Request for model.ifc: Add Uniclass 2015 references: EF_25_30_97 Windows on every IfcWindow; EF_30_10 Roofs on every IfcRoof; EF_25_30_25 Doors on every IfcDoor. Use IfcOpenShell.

First a look at what the model holds.

```python
import ifcopenshell

model = ifcopenshell.open("model.ifc")
print(model.schema)
print("classifications:", [c.Name for c in model.by_type("IfcClassification")])
for ifc_class in ("IfcDoor", "IfcRoof", "IfcStair", "IfcWall", "IfcWindow"):
    print(ifc_class, len(model.by_type(ifc_class)))
```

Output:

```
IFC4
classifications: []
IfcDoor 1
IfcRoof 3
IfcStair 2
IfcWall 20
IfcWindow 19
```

```python
import ifcopenshell
import ifcopenshell.api.classification

model = ifcopenshell.open("model.ifc")

system = ifcopenshell.api.classification.add_classification(model, classification="Uniclass 2015")

codes = {
    "IfcWindow": ("EF_25_30_97", "Windows"),
    "IfcRoof": ("EF_30_10", "Roofs"),
    "IfcDoor": ("EF_25_30_25", "Doors"),
}
for ifc_class, (code, name) in codes.items():
    products = model.by_type(ifc_class)
    ifcopenshell.api.classification.add_reference(
        model, products=products, classification=system, identification=code, name=name
    )
    print(code, len(products))

model.write("model_v2.ifc")
```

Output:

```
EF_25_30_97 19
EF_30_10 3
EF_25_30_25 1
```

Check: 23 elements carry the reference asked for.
